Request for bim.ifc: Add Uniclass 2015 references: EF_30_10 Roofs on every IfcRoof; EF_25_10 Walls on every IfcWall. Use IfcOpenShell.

First a look at what the model holds.

```python
import ifcopenshell

model = ifcopenshell.open("bim.ifc")
print(model.schema)
print("classifications:", [c.Name for c in model.by_type("IfcClassification")])
for ifc_class in ("IfcDoor", "IfcRoof", "IfcStair", "IfcWall", "IfcWindow"):
    print(ifc_class, len(model.by_type(ifc_class)))
```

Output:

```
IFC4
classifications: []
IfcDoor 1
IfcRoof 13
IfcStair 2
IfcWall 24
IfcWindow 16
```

```python
import ifcopenshell
import ifcopenshell.api.classification

model = ifcopenshell.open("bim.ifc")

system = ifcopenshell.api.classification.add_classification(model, classification="Uniclass 2015")

codes = {
    "IfcRoof": ("EF_30_10", "Roofs"),
    "IfcWall": ("EF_25_10", "Walls"),
}
for ifc_class, (code, name) in codes.items():
    products = model.by_type(ifc_class)
    ifcopenshell.api.classification.add_reference(
        model, products=products, classification=system, identification=code, name=name
    )
    print(code, len(products))

model.write("bim_updated.ifc")
```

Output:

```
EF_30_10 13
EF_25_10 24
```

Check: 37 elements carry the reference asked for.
